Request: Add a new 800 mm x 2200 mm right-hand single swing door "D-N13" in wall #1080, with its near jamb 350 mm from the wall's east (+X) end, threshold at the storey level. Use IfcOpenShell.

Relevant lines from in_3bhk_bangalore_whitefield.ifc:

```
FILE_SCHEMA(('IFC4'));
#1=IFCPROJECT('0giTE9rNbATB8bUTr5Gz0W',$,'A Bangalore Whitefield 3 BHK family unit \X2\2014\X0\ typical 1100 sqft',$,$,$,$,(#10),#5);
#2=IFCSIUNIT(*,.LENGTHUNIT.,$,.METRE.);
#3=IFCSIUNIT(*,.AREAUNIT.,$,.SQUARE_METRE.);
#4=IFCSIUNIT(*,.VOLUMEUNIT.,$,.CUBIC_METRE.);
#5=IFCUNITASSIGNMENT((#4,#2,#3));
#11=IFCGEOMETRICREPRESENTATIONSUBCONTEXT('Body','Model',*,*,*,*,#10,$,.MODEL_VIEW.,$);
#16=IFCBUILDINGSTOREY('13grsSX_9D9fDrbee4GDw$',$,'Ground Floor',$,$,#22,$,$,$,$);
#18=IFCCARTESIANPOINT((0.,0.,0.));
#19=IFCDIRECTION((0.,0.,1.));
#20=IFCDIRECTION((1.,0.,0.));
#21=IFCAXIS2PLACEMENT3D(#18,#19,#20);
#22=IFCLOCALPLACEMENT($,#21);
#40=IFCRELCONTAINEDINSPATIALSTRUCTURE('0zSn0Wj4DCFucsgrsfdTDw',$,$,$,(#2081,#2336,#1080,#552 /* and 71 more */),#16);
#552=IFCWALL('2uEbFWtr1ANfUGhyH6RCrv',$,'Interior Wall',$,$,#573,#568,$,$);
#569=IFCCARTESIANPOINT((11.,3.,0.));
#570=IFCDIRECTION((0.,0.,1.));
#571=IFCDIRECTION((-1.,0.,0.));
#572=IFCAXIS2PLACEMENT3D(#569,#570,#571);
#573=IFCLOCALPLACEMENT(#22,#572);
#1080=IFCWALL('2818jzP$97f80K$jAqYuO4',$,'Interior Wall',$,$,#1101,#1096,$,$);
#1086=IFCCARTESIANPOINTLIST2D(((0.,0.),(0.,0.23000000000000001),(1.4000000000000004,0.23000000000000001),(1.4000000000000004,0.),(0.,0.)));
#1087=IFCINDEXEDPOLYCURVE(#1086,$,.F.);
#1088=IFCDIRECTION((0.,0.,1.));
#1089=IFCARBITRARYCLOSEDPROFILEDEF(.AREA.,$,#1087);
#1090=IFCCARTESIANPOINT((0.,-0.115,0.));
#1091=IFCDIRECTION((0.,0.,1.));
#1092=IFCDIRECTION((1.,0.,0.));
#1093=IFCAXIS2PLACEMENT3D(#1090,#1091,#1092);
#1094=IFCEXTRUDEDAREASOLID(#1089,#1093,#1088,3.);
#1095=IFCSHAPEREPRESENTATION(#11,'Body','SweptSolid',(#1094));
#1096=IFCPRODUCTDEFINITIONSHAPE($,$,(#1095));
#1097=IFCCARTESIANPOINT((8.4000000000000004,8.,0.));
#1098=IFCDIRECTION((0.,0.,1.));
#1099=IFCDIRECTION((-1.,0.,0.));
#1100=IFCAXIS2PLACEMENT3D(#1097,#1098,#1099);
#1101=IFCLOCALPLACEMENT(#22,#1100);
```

```python
import numpy as np
import ifcopenshell
import ifcopenshell.api.feature
import ifcopenshell.api.geometry
import ifcopenshell.api.root
import ifcopenshell.api.spatial
import ifcopenshell.geom
import ifcopenshell.util.element
import ifcopenshell.util.placement
import ifcopenshell.util.representation
import ifcopenshell.util.shape
import ifcopenshell.util.unit

model = ifcopenshell.open("in_3bhk_bangalore_whitefield.ifc")
unit_scale = ifcopenshell.util.unit.calculate_unit_scale(model)
settings = ifcopenshell.geom.settings()


def volume(element):
    """Net volume in cubic metres, openings subtracted."""
    shape = ifcopenshell.geom.create_shape(settings, element)
    return ifcopenshell.util.shape.get_volume(shape.geometry)


wall = model.by_guid("2818jzP$97f80K$jAqYuO4")
storey = ifcopenshell.util.element.get_container(wall, ifc_class="IfcBuildingStorey")
context = ifcopenshell.util.representation.get_context(model, "Model", "Body", "MODEL_VIEW")
before = volume(wall)

width, height, from_end, sill = 0.8, 2.2, 0.35, 0.0  # metres

# The wall runs along its own X axis, and the end named is its -X end.
wall_shape = ifcopenshell.geom.create_shape(settings, wall)
x, y, z = ifcopenshell.util.shape.get_vertices(wall_shape.geometry).T
start = x.min() + from_end
face, thickness = float(y.min()), float(y.max() - y.min())
wall_matrix = ifcopenshell.util.placement.get_local_placement(wall.ObjectPlacement)
level = ifcopenshell.util.placement.get_local_placement(storey.ObjectPlacement)[2, 3]


def in_wall(x, y):
    """Placement at x, y metres in the wall's axes, at sill height."""
    matrix = wall_matrix.copy()
    matrix[:, 3] = wall_matrix @ np.array([x / unit_scale, y / unit_scale, 0.0, 1.0])
    matrix[2, 3] = level + sill / unit_scale
    return matrix


# Opening: a box that overshoots both wall faces by 50 mm.
opening = ifcopenshell.api.root.create_entity(model, ifc_class="IfcOpeningElement", predefined_type="OPENING")
box = ifcopenshell.api.geometry.add_wall_representation(
    model, context=context, length=width, height=height, thickness=thickness + 0.1
)
ifcopenshell.api.geometry.assign_representation(model, product=opening, representation=box)
ifcopenshell.api.geometry.edit_object_placement(model, product=opening, matrix=in_wall(start, face - 0.05), is_si=False)
ifcopenshell.api.feature.add_feature(model, feature=opening, element=wall)

door = ifcopenshell.api.root.create_entity(model, ifc_class="IfcDoor", name="D-N13", predefined_type="DOOR")
door.OverallWidth, door.OverallHeight = width / unit_scale, height / unit_scale
door.OperationType = "SINGLE_SWING_RIGHT"
body = ifcopenshell.api.geometry.add_door_representation(
    model,
    context=context,
    overall_width=door.OverallWidth,
    overall_height=door.OverallHeight,
    operation_type="SINGLE_SWING_RIGHT",
    lining_properties={"LiningDepth": thickness / unit_scale, "ThresholdDepth": thickness / unit_scale},
)
ifcopenshell.api.geometry.assign_representation(model, product=door, representation=body)
ifcopenshell.api.spatial.assign_container(model, products=[door], relating_structure=storey)
ifcopenshell.api.feature.add_filling(model, opening=opening, element=door)

# The lining spans the wall, so the door starts at the wall face.
ifcopenshell.api.geometry.edit_object_placement(model, product=door, matrix=in_wall(start, face), is_si=False)

after = volume(wall)

print(f"wall volume {before:.3f} -> {after:.3f} m3")

model.write("in_3bhk_bangalore_whitefield_rev.ifc")
```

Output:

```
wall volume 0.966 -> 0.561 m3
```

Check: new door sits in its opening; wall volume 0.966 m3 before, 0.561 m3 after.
